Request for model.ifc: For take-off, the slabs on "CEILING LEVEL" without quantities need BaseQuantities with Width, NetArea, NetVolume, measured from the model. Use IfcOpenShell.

First a look at what the model holds.

```python
import ifcopenshell
import ifcopenshell.util.element
import ifcopenshell.util.unit

model = ifcopenshell.open("model.ifc")
print(model.schema)
for unit_type in ("LENGTHUNIT", "AREAUNIT", "VOLUMEUNIT"):
    print(unit_type, ifcopenshell.util.unit.calculate_unit_scale(model, unit_type))
storey = next(s for s in model.by_type("IfcBuildingStorey") if s.Name == "CEILING LEVEL")
slabs = [e for e in ifcopenshell.util.element.get_decomposition(storey) if e.is_a("IfcSlab")]
for e in sorted(slabs, key=lambda e: e.id()):
    print(e.id(), e.is_a(), e.Name, list(ifcopenshell.util.element.get_psets(e, qtos_only=True)), sep=" | ")
```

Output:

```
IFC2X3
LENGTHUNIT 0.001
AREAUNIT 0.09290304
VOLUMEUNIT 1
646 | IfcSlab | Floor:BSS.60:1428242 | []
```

```python
import ifcopenshell
import ifcopenshell.api.pset
import ifcopenshell.geom
import ifcopenshell.util.element
import ifcopenshell.util.shape
import ifcopenshell.util.unit

model = ifcopenshell.open("model.ifc")
unit_scale = ifcopenshell.util.unit.calculate_unit_scale(model)
area_scale = ifcopenshell.util.unit.calculate_unit_scale(model, "AREAUNIT")
volume_scale = ifcopenshell.util.unit.calculate_unit_scale(model, "VOLUMEUNIT")
settings = ifcopenshell.geom.settings()

storey = next(s for s in model.by_type("IfcBuildingStorey") if s.Name == "CEILING LEVEL")
slabs = [e for e in ifcopenshell.util.element.get_decomposition(storey) if e.is_a("IfcSlab")]

for e in sorted(slabs, key=lambda e: e.id()):
    if ifcopenshell.util.element.get_psets(e, qtos_only=True, should_inherit=False):
        continue
    # Geometry comes back in metres, in the element's own axes.
    shape = ifcopenshell.geom.create_shape(settings, e)
    values = {
        "Width": ifcopenshell.util.shape.get_z(shape.geometry) / unit_scale,
        "NetArea": ifcopenshell.util.shape.get_footprint_area(shape.geometry) / area_scale,
        "NetVolume": ifcopenshell.util.shape.get_volume(shape.geometry) / volume_scale,
    }
    qto = ifcopenshell.api.pset.add_qto(model, product=e, name="BaseQuantities")
    ifcopenshell.api.pset.edit_qto(model, qto=qto, properties=values)
    print(e.id(), {k: round(v, 3) for k, v in values.items()})

model.write("model_v2.ifc")
```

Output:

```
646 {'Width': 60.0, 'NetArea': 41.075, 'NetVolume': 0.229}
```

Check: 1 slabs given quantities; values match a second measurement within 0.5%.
